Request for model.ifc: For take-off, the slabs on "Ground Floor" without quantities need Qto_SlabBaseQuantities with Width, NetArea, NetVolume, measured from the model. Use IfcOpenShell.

First a look at what the model holds.

```python
import ifcopenshell
import ifcopenshell.util.element
import ifcopenshell.util.unit

model = ifcopenshell.open("model.ifc")
print(model.schema)
for unit_type in ("LENGTHUNIT", "AREAUNIT", "VOLUMEUNIT"):
    print(unit_type, ifcopenshell.util.unit.calculate_unit_scale(model, unit_type))
storey = next(s for s in model.by_type("IfcBuildingStorey") if s.Name == "Ground Floor")
slabs = [e for e in ifcopenshell.util.element.get_decomposition(storey) if e.is_a("IfcSlab")]
for e in sorted(slabs, key=lambda e: e.id()):
    print(e.id(), e.is_a(), e.Name, list(ifcopenshell.util.element.get_psets(e, qtos_only=True)), sep=" | ")
```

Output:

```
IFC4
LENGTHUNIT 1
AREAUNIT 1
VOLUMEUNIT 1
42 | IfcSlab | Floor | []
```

```python
import ifcopenshell
import ifcopenshell.api.pset
import ifcopenshell.geom
import ifcopenshell.util.element
import ifcopenshell.util.shape
import ifcopenshell.util.unit

model = ifcopenshell.open("model.ifc")
unit_scale = ifcopenshell.util.unit.calculate_unit_scale(model)
area_scale = ifcopenshell.util.unit.calculate_unit_scale(model, "AREAUNIT")
volume_scale = ifcopenshell.util.unit.calculate_unit_scale(model, "VOLUMEUNIT")
settings = ifcopenshell.geom.settings()

storey = next(s for s in model.by_type("IfcBuildingStorey") if s.Name == "Ground Floor")
slabs = [e for e in ifcopenshell.util.element.get_decomposition(storey) if e.is_a("IfcSlab")]

for e in sorted(slabs, key=lambda e: e.id()):
    if ifcopenshell.util.element.get_psets(e, qtos_only=True, should_inherit=False):
        continue
    # Geometry comes back in metres, in the element's own axes.
    shape = ifcopenshell.geom.create_shape(settings, e)
    values = {
        "Width": ifcopenshell.util.shape.get_z(shape.geometry) / unit_scale,
        "NetArea": ifcopenshell.util.shape.get_footprint_area(shape.geometry) / area_scale,
        "NetVolume": ifcopenshell.util.shape.get_volume(shape.geometry) / volume_scale,
    }
    qto = ifcopenshell.api.pset.add_qto(model, product=e, name="Qto_SlabBaseQuantities")
    ifcopenshell.api.pset.edit_qto(model, qto=qto, properties=values)
    print(e.id(), {k: round(v, 3) for k, v in values.items()})

model.write("model_updated.ifc")
```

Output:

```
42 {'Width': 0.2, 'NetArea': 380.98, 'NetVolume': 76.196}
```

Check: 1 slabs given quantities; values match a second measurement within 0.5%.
